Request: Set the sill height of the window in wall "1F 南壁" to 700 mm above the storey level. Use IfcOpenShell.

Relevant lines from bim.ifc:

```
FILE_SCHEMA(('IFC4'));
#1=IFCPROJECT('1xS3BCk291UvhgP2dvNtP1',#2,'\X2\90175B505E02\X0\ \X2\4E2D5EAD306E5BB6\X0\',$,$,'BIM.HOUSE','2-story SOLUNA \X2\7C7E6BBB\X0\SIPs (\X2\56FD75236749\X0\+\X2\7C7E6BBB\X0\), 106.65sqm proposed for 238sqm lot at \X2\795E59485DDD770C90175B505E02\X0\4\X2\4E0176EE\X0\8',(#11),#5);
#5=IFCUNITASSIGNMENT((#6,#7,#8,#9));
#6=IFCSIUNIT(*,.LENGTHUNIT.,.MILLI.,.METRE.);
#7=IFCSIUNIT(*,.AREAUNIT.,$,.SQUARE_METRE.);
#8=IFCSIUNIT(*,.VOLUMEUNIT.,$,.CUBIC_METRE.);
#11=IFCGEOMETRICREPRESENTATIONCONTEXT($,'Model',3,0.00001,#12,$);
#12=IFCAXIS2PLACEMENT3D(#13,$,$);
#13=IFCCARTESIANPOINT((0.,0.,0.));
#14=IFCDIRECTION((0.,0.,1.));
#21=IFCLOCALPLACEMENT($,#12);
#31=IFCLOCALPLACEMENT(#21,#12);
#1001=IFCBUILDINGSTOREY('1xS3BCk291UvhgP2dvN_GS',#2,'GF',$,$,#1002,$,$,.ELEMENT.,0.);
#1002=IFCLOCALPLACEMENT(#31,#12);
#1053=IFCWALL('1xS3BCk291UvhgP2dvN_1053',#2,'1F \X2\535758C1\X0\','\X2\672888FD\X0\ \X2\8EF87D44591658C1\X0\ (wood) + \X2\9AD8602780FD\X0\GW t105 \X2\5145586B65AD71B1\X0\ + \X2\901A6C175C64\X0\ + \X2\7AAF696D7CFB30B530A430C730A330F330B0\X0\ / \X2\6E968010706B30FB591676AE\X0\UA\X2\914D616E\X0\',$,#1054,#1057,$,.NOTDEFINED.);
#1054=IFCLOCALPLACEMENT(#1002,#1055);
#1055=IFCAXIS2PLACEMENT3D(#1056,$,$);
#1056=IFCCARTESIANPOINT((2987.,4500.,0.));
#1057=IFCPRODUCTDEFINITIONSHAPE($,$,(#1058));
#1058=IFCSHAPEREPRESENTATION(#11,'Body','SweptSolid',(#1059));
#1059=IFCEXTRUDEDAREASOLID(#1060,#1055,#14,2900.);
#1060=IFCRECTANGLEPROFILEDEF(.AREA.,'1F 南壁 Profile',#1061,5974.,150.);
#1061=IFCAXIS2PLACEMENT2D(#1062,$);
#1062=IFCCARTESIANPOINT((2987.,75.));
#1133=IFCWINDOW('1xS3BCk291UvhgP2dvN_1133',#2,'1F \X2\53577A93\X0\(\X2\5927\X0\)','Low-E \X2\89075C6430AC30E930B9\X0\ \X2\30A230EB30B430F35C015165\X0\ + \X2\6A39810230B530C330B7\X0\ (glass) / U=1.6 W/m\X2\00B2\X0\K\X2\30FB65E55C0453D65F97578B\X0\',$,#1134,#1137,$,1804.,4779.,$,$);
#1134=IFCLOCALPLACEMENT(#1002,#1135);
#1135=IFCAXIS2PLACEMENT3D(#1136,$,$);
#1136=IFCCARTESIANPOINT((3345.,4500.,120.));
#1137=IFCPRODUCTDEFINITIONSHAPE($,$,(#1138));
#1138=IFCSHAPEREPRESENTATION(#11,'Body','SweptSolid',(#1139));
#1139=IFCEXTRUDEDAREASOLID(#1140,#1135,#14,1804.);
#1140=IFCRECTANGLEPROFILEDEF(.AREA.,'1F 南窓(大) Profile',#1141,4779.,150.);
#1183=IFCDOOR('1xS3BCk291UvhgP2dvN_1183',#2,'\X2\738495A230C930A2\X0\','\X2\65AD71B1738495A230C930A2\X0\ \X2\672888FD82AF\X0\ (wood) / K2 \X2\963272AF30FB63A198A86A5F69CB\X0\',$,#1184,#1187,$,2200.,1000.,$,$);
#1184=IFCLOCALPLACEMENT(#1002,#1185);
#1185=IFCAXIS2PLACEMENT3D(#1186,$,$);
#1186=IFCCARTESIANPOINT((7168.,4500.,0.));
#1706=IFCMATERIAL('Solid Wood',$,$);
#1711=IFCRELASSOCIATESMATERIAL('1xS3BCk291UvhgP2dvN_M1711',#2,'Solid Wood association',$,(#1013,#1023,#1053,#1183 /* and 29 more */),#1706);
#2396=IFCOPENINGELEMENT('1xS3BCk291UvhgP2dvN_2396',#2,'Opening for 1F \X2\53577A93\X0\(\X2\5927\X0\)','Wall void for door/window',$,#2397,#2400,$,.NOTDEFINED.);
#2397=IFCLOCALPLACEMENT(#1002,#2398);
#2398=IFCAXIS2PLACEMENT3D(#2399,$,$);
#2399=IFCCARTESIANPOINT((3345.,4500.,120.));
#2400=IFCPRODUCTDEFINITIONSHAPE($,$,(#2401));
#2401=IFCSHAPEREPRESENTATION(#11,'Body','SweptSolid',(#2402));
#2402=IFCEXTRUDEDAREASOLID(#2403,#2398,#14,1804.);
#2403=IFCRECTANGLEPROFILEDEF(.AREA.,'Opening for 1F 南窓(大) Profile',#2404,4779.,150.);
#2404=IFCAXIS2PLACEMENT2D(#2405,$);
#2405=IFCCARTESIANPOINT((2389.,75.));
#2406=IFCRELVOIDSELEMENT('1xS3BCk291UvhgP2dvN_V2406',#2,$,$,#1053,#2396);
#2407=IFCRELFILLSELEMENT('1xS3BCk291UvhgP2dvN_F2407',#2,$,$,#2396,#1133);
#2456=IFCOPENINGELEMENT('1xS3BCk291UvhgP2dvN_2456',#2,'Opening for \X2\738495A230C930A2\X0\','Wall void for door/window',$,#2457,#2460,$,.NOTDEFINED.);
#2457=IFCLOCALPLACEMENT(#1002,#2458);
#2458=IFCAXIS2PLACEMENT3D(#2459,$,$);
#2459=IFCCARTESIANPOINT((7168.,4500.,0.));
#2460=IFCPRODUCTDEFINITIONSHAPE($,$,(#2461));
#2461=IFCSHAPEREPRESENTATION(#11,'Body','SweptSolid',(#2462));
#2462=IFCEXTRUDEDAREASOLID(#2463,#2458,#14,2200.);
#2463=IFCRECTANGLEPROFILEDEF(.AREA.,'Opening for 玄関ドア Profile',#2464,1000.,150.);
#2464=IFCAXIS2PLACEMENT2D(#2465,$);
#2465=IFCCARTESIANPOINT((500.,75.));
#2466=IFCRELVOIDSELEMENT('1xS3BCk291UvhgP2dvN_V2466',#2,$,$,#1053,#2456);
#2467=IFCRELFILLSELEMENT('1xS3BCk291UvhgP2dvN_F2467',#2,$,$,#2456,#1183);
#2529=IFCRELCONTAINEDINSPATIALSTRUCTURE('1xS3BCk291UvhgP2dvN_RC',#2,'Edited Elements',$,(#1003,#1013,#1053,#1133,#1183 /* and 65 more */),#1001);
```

```python
import numpy as np
import ifcopenshell
import ifcopenshell.api.geometry
import ifcopenshell.geom
import ifcopenshell.util.element
import ifcopenshell.util.placement
import ifcopenshell.util.shape
import ifcopenshell.util.unit

model = ifcopenshell.open("bim.ifc")
unit_scale = ifcopenshell.util.unit.calculate_unit_scale(model)

window = model.by_guid("1xS3BCk291UvhgP2dvN_1133")
opening = window.FillsVoids[0].RelatingOpeningElement
storey = ifcopenshell.util.element.get_container(window, ifc_class="IfcBuildingStorey")
level = ifcopenshell.util.placement.get_local_placement(storey.ObjectPlacement)[2, 3]

# The opening's origin need not be at the sill, so measure its lowest point.
shape = ifcopenshell.geom.create_shape(ifcopenshell.geom.settings(), opening)
bottom = ifcopenshell.util.shape.get_shape_bottom_elevation(shape, shape.geometry) / unit_scale
dz = level + 0.7 / unit_scale - bottom

shift = np.array([0.0, 0.0, dz])
# The window is not placed relative to its opening, so move both.
for product in (opening, window):
    matrix = ifcopenshell.util.placement.get_local_placement(product.ObjectPlacement)
    matrix[:3, 3] += shift
    ifcopenshell.api.geometry.edit_object_placement(model, product=product, matrix=matrix, is_si=False)

print(f"moved by {dz * unit_scale:+.3f} m")

model.write("bim_updated.ifc")
```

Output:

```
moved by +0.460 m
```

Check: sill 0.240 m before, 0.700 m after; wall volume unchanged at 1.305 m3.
